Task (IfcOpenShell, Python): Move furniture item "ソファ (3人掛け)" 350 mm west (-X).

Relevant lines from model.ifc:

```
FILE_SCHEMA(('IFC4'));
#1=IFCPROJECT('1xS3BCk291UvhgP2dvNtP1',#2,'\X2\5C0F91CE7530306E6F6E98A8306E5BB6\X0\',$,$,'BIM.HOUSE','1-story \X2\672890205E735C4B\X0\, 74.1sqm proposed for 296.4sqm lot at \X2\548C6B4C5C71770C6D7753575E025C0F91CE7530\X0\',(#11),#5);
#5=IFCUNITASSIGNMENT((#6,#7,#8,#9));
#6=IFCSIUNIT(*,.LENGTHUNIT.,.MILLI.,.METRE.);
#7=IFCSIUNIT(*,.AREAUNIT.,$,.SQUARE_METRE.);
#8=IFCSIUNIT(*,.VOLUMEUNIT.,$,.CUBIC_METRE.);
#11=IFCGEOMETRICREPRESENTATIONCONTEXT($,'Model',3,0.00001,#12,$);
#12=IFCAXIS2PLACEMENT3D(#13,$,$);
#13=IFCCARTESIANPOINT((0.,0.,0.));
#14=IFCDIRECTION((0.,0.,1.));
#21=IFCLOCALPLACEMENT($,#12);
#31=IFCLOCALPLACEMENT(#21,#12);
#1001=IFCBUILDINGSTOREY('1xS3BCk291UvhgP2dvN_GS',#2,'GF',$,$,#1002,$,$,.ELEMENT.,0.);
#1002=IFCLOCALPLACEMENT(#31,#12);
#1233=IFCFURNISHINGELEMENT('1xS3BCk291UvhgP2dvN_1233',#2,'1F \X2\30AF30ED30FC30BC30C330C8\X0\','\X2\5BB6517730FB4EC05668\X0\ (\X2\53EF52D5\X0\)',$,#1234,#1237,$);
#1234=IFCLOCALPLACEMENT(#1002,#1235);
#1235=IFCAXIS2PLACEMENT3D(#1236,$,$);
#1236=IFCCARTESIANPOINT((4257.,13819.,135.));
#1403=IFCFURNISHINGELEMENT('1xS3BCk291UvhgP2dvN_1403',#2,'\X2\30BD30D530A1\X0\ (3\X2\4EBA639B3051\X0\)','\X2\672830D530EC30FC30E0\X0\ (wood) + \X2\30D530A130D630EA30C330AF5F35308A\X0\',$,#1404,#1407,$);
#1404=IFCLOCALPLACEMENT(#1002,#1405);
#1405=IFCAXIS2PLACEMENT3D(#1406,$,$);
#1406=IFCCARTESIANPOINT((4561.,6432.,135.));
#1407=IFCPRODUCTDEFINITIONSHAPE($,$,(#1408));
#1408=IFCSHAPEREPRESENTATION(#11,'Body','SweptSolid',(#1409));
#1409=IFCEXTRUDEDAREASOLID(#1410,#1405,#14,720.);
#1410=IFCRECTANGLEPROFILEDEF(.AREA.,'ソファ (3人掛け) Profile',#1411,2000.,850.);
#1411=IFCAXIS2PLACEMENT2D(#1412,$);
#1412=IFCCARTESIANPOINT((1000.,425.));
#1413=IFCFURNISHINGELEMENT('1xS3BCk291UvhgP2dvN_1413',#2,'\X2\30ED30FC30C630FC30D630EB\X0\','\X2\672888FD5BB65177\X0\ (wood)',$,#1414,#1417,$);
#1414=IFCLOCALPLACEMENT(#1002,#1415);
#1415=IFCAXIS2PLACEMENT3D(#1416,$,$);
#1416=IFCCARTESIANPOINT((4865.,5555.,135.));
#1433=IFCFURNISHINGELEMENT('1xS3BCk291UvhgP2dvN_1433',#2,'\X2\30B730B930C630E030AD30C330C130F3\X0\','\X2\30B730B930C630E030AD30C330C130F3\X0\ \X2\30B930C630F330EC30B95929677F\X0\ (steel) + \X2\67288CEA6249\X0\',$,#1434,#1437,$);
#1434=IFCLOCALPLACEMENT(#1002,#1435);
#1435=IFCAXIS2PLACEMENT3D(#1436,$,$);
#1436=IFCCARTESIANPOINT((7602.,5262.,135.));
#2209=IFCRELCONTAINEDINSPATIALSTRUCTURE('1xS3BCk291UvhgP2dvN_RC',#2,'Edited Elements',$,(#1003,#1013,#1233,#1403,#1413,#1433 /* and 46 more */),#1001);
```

```python
import ifcopenshell
import ifcopenshell.api.geometry
import ifcopenshell.util.placement
import ifcopenshell.util.unit

model = ifcopenshell.open("model.ifc")
unit_scale = ifcopenshell.util.unit.calculate_unit_scale(model)

item = model.by_id(1403)
matrix = ifcopenshell.util.placement.get_local_placement(item.ObjectPlacement)
matrix[0, 3] -= 0.35 / unit_scale
ifcopenshell.api.geometry.edit_object_placement(model, product=item, matrix=matrix, is_si=False)

print(ifcopenshell.util.placement.get_local_placement(item.ObjectPlacement).round(3) + 0.0)

model.write("model_v2.ifc")
```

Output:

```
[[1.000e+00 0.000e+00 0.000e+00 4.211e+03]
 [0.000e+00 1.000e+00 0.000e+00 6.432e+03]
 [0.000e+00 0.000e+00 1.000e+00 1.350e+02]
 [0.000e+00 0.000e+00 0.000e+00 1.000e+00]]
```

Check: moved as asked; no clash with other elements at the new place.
